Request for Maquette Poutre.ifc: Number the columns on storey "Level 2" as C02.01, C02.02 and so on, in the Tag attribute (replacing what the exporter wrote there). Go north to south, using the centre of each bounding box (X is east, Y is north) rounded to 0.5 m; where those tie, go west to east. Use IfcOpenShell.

First a look at what the model holds.

```python
import ifcopenshell
import ifcopenshell.util.element
import ifcopenshell.util.placement

model = ifcopenshell.open("Maquette Poutre.ifc")
print(model.schema)
storey = next(s for s in model.by_type("IfcBuildingStorey") if s.Name == "Level 2")
columns = [e for e in ifcopenshell.util.element.get_decomposition(storey) if e.is_a("IfcColumn")]
for e in sorted(columns, key=lambda e: e.id()):
    origin = ifcopenshell.util.placement.get_local_placement(e.ObjectPlacement)[:3, 3]
    print(e.id(), e.Tag, e.Name, origin.round(2) + 0.0, sep=" | ")
```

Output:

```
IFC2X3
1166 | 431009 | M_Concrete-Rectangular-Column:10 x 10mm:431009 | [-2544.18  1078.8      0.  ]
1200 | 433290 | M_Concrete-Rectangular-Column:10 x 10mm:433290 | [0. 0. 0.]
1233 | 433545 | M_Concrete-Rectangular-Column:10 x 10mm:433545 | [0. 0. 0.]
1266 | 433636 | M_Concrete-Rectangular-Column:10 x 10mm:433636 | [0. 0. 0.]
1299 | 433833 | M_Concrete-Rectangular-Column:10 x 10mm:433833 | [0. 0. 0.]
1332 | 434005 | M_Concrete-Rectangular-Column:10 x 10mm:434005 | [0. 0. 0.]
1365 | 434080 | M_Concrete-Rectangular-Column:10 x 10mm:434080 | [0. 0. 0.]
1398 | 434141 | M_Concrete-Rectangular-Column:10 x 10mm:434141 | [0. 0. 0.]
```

```python
import ifcopenshell
import ifcopenshell.geom
import ifcopenshell.util.element
import ifcopenshell.util.shape

model = ifcopenshell.open("Maquette Poutre.ifc")
settings = ifcopenshell.geom.settings()
settings.set("use-world-coords", True)


def centre(element):
    shape = ifcopenshell.geom.create_shape(settings, element)
    return ifcopenshell.util.shape.get_bbox_centroid(shape.geometry)


storey = next(s for s in model.by_type("IfcBuildingStorey") if s.Name == "Level 2")
columns = [e for e in ifcopenshell.util.element.get_decomposition(storey) if e.is_a("IfcColumn")]

# Insertion points can sit at a corner or the storey origin, so sort by the geometry (in metres).
centres = {e: centre(e) for e in columns}
columns.sort(key=lambda e: (-round(centres[e][1] / 0.5), centres[e][0]))

for i, e in enumerate(columns, start=1):
    number = f"C02.{i:02d}"
    e.Tag = number
    print(e.id(), number)

model.write("Maquette Poutre_rev.ifc")
```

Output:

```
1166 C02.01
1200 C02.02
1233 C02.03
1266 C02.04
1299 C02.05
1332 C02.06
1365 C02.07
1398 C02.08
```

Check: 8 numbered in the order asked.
